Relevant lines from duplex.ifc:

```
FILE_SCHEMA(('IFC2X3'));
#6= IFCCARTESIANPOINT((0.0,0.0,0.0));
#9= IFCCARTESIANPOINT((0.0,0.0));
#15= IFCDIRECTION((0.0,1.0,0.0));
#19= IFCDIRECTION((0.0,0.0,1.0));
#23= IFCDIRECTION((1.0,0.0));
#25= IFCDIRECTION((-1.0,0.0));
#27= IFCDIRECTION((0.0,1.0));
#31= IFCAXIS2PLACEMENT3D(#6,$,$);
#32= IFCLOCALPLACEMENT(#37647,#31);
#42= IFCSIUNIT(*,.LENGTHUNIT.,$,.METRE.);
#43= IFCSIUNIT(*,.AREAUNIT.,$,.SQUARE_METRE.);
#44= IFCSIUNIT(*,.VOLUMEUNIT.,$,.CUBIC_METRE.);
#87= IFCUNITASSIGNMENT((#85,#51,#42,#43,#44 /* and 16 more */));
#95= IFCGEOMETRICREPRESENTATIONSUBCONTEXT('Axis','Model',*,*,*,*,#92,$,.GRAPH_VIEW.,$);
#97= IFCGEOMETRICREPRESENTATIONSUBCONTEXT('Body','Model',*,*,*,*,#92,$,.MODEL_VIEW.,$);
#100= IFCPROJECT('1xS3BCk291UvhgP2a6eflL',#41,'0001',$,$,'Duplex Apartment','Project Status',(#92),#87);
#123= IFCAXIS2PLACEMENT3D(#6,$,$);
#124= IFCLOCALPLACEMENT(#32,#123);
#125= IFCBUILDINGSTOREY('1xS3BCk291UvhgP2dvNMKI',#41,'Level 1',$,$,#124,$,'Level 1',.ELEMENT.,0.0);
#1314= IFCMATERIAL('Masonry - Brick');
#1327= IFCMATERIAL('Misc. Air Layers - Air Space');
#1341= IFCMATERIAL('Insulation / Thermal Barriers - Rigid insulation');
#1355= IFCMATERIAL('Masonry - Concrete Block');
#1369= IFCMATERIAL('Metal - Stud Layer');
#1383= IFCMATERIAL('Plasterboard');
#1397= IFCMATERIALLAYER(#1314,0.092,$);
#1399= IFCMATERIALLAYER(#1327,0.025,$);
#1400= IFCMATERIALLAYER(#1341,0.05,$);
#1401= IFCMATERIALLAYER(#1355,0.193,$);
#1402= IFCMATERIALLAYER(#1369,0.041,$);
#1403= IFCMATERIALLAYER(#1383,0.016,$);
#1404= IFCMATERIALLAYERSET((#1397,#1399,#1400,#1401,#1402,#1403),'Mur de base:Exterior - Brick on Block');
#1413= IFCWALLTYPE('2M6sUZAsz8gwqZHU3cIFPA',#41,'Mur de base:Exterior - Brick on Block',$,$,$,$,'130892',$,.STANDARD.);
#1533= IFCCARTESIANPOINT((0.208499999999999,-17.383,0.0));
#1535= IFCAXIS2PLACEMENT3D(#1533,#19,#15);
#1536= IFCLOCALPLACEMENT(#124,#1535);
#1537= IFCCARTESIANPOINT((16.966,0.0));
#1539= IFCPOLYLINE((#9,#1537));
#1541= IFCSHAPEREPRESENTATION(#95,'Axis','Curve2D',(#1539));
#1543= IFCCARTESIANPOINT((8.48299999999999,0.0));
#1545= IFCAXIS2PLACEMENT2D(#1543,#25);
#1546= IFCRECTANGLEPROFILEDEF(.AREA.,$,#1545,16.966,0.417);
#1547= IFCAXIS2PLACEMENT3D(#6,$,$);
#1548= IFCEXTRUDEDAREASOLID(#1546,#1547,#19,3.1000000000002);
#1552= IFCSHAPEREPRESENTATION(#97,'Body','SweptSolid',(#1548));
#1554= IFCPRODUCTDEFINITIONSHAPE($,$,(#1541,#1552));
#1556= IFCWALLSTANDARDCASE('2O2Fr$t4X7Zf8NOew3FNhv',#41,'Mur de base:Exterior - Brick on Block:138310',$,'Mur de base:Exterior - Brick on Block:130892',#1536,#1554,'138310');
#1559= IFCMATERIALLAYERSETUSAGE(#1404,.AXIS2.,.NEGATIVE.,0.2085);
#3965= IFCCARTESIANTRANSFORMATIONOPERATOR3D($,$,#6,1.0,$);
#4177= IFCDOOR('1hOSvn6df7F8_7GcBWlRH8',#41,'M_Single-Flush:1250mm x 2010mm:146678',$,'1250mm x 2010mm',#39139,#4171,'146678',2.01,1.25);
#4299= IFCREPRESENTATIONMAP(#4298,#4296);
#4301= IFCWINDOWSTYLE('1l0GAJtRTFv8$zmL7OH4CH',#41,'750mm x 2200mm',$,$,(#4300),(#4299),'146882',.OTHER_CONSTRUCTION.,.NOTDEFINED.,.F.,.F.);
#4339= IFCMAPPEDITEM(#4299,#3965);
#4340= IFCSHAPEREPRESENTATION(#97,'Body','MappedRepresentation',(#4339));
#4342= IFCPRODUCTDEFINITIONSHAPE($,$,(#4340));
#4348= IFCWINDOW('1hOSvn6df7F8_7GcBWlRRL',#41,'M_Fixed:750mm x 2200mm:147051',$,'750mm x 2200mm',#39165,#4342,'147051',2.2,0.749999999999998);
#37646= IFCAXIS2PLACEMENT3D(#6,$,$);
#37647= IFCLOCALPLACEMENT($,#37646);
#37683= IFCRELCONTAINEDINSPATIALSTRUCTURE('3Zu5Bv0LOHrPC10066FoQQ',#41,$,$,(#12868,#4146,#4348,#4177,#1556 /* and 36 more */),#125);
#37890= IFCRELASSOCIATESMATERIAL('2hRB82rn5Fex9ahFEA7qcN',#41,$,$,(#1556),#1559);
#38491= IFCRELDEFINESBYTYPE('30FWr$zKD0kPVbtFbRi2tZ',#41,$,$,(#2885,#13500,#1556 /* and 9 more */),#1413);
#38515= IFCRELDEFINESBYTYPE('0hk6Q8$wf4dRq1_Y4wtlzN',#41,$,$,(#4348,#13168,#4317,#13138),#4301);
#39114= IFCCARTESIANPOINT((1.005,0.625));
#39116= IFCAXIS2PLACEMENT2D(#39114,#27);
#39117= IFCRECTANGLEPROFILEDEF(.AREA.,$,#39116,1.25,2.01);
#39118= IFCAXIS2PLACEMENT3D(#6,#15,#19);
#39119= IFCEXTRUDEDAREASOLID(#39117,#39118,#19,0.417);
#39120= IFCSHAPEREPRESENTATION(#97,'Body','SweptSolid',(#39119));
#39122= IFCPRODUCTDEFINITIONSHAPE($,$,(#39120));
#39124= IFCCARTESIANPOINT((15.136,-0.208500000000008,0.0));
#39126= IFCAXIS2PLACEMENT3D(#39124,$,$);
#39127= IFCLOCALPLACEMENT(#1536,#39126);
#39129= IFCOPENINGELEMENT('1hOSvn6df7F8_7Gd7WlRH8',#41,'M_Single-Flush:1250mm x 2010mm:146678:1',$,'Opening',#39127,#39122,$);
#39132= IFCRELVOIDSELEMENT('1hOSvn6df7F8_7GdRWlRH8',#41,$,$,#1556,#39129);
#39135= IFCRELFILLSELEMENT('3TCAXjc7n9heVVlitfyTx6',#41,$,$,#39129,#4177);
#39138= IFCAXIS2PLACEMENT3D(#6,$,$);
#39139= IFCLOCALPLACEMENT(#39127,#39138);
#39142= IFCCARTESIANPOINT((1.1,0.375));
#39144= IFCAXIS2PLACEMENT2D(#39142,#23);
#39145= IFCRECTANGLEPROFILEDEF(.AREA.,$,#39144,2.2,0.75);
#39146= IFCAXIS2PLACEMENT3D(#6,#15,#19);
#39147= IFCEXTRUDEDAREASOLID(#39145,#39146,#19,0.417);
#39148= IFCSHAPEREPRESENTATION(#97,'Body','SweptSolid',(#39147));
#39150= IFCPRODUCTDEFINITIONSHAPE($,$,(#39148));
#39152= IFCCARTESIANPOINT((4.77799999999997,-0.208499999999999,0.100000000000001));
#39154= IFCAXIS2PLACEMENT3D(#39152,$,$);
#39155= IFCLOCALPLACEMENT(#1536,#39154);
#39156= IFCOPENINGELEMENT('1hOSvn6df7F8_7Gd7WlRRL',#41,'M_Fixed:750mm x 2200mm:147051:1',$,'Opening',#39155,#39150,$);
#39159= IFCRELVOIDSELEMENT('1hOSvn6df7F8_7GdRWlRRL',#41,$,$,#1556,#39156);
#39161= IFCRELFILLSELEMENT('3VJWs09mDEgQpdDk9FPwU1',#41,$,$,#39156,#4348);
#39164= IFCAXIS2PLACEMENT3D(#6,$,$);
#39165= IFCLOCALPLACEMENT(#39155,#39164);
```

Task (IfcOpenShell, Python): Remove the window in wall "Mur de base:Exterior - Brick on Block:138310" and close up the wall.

```python
import ifcopenshell
import ifcopenshell.api.feature
import ifcopenshell.api.root
import ifcopenshell.geom
import ifcopenshell.util.shape

model = ifcopenshell.open("duplex.ifc")
settings = ifcopenshell.geom.settings()


def volume(element):
    """Net volume in cubic metres, openings subtracted."""
    shape = ifcopenshell.geom.create_shape(settings, element)
    return ifcopenshell.util.shape.get_volume(shape.geometry)


window = model.by_guid("1hOSvn6df7F8_7GcBWlRRL")
opening = window.FillsVoids[0].RelatingOpeningElement
wall = opening.VoidsElements[0].RelatingBuildingElement
before = volume(wall)

ifcopenshell.api.root.remove_product(model, product=window)
ifcopenshell.api.feature.remove_feature(model, feature=opening)

after = volume(wall)

print(f"wall volume {before:.3f} -> {after:.3f} m3")

model.write("duplex_rev.ifc")
```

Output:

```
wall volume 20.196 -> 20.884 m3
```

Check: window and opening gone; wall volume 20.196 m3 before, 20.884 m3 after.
